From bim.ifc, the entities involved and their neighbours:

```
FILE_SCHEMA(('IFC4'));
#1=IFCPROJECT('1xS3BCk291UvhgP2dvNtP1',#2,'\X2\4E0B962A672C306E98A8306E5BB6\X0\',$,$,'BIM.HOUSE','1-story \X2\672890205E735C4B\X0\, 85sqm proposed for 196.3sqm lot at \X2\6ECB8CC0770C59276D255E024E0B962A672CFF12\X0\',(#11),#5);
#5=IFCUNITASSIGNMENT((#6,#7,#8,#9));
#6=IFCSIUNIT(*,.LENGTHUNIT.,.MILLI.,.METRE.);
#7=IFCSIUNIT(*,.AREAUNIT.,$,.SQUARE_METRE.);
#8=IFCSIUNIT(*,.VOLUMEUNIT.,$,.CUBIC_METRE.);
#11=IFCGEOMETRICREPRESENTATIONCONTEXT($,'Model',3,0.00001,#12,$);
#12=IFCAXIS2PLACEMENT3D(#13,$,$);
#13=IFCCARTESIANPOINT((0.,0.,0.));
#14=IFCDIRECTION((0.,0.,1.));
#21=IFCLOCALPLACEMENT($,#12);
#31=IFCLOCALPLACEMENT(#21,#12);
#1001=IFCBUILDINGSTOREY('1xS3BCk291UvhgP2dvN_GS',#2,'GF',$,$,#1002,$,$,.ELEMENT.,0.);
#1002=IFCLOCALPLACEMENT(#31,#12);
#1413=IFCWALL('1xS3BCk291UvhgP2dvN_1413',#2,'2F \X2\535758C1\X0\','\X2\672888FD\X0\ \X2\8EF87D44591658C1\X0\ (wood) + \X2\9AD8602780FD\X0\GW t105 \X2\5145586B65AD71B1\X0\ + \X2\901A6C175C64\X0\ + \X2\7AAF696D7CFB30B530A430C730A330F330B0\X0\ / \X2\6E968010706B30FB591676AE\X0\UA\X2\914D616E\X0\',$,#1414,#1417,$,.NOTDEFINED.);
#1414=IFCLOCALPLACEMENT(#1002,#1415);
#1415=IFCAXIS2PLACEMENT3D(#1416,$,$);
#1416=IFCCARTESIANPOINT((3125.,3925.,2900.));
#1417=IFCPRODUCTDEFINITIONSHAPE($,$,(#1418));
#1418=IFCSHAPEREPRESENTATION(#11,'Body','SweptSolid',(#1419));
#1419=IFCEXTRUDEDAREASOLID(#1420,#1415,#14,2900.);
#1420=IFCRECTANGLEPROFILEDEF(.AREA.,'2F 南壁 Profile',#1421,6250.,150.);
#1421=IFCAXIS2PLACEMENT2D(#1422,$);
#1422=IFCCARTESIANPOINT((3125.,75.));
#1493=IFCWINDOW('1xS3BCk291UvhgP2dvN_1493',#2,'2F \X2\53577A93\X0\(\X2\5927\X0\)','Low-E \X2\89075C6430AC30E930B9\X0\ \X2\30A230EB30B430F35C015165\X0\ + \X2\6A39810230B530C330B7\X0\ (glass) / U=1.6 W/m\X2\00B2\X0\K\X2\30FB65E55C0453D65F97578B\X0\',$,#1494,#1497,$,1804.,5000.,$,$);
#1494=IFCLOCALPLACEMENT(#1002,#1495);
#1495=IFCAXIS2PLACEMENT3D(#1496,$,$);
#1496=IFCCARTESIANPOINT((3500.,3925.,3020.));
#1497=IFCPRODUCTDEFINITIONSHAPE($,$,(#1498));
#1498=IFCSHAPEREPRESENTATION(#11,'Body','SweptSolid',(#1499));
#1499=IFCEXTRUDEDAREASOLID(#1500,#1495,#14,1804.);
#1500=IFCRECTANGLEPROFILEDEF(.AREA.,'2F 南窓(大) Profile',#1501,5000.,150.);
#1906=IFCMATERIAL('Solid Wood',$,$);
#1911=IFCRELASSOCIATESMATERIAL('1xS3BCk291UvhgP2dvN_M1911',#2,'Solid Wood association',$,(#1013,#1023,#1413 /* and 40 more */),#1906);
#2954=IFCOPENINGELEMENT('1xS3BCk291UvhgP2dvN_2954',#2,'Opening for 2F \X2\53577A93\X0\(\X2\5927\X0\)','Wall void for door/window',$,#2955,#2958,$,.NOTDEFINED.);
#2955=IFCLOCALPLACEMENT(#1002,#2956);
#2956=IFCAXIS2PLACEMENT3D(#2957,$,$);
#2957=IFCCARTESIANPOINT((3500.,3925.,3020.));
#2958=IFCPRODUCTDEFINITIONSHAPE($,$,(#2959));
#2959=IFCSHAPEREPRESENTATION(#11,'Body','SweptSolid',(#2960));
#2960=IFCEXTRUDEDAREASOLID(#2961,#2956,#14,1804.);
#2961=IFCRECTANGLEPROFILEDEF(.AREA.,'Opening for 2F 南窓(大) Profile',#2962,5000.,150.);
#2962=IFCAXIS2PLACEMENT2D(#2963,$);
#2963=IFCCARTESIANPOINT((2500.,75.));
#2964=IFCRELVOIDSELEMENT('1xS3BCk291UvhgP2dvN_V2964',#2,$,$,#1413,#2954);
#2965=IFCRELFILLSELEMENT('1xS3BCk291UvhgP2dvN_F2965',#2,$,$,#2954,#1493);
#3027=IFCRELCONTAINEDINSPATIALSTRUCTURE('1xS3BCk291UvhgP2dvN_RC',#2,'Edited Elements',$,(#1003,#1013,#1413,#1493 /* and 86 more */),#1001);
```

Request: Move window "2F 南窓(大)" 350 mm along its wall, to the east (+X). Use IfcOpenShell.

```python
import ifcopenshell
import ifcopenshell.api.geometry
import ifcopenshell.util.placement

model = ifcopenshell.open("bim.ifc")

window = model.by_guid("1xS3BCk291UvhgP2dvN_1493")
opening = window.FillsVoids[0].RelatingOpeningElement
wall = opening.VoidsElements[0].RelatingBuildingElement

wall_matrix = ifcopenshell.util.placement.get_local_placement(wall.ObjectPlacement)
shift = wall_matrix[:3, 0] * 350.0
before = ifcopenshell.util.placement.get_local_placement(window.ObjectPlacement)[:3, 3].copy()

# The window is not placed relative to its opening, so move both.
for product in (opening, window):
    matrix = ifcopenshell.util.placement.get_local_placement(product.ObjectPlacement)
    matrix[:3, 3] += shift
    ifcopenshell.api.geometry.edit_object_placement(model, product=product, matrix=matrix, is_si=False)

after = ifcopenshell.util.placement.get_local_placement(window.ObjectPlacement)[:3, 3]
print("window moved by", (after - before).round(3) + 0.0)

model.write("bim_edited.ifc")
```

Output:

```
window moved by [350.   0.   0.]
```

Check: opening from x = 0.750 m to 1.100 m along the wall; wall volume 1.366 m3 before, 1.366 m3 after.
